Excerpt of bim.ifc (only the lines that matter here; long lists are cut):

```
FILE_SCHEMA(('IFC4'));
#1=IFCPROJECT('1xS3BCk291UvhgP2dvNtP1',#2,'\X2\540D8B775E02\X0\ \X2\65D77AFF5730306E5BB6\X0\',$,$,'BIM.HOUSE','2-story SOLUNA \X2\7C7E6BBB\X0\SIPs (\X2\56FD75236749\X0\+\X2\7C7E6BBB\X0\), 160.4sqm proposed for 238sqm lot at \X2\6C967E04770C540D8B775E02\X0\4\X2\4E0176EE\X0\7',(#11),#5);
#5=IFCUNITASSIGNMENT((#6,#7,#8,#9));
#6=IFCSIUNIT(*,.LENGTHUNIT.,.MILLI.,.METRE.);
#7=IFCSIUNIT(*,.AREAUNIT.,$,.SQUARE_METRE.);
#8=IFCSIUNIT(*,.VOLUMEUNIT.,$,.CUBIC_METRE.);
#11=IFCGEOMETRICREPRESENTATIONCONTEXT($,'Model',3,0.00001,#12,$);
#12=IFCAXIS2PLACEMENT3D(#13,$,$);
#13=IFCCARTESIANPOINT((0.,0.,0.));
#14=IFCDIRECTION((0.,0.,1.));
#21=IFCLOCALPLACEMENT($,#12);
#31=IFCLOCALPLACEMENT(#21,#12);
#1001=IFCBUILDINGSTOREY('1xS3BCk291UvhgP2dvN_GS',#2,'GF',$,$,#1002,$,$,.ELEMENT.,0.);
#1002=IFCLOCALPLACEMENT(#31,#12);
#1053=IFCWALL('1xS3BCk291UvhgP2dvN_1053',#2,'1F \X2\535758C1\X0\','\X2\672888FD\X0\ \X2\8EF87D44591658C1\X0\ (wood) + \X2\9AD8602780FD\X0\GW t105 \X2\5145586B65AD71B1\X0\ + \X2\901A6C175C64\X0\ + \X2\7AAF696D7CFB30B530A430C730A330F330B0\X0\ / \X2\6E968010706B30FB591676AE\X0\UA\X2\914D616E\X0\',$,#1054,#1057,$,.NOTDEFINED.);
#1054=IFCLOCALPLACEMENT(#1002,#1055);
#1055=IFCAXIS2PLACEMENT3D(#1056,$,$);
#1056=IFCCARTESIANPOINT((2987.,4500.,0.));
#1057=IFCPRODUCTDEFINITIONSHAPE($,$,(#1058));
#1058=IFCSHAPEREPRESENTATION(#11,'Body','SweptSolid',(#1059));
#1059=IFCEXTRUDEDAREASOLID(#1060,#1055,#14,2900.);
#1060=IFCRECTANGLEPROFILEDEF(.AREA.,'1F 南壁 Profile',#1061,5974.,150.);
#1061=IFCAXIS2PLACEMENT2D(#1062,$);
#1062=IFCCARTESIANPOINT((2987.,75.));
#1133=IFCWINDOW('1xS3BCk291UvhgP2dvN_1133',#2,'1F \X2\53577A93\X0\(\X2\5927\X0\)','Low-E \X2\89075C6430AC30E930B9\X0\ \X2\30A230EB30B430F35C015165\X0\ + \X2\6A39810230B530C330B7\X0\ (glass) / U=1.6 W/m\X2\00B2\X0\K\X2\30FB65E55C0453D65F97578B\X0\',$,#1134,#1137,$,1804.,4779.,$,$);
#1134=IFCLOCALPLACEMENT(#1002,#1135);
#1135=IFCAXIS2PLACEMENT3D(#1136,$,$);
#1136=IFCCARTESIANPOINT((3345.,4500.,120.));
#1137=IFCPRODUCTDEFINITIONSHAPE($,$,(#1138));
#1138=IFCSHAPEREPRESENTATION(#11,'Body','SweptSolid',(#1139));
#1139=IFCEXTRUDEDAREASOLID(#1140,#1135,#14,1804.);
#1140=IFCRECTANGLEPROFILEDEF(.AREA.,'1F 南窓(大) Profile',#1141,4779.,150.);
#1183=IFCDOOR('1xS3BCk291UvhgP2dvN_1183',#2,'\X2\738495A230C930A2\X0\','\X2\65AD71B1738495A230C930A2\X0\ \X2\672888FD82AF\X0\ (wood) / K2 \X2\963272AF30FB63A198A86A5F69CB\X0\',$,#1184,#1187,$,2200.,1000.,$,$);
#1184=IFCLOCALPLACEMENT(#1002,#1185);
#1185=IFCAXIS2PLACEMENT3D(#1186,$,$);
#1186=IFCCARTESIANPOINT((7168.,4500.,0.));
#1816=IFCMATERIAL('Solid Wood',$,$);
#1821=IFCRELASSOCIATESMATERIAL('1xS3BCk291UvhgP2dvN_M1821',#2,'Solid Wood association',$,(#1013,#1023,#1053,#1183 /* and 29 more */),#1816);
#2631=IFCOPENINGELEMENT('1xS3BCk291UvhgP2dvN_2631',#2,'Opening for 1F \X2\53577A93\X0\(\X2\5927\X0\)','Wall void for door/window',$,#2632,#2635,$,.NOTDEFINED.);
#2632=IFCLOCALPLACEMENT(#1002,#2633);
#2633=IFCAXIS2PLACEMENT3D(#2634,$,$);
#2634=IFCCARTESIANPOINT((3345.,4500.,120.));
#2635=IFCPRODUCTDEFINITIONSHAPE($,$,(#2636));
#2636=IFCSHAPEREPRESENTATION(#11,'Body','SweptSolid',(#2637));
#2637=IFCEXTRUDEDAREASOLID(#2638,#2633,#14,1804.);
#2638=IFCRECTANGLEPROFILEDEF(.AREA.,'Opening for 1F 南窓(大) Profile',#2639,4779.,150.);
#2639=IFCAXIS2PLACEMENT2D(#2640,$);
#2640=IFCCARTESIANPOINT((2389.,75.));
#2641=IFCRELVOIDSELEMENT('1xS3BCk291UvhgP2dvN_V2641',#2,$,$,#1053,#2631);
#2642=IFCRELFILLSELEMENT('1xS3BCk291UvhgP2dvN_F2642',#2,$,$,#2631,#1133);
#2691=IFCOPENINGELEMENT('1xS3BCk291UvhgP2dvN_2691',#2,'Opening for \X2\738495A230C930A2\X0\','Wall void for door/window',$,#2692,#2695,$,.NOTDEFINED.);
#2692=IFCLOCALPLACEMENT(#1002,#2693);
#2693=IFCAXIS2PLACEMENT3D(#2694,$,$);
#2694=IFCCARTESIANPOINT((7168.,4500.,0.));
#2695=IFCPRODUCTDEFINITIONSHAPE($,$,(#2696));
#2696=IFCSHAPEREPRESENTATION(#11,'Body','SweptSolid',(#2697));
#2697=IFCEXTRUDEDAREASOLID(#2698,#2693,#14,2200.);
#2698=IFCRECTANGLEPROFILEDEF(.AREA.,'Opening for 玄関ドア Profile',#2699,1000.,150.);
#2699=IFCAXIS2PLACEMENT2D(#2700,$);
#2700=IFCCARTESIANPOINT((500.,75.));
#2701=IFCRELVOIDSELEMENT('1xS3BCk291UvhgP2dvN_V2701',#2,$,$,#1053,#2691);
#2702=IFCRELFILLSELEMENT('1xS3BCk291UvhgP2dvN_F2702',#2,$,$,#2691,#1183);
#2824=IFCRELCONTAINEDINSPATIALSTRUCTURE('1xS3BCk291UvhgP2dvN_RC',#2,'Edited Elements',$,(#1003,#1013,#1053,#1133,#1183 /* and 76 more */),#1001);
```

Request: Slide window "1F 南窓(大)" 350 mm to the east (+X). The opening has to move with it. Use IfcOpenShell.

```python
import ifcopenshell
import ifcopenshell.api.geometry
import ifcopenshell.util.placement

model = ifcopenshell.open("bim.ifc")

window = model.by_guid("1xS3BCk291UvhgP2dvN_1133")
opening = window.FillsVoids[0].RelatingOpeningElement
wall = opening.VoidsElements[0].RelatingBuildingElement

wall_matrix = ifcopenshell.util.placement.get_local_placement(wall.ObjectPlacement)
shift = wall_matrix[:3, 0] * 350.0
before = ifcopenshell.util.placement.get_local_placement(window.ObjectPlacement)[:3, 3].copy()

# The window is not placed relative to its opening, so move both.
for product in (opening, window):
    matrix = ifcopenshell.util.placement.get_local_placement(product.ObjectPlacement)
    matrix[:3, 3] += shift
    ifcopenshell.api.geometry.edit_object_placement(model, product=product, matrix=matrix, is_si=False)

after = ifcopenshell.util.placement.get_local_placement(window.ObjectPlacement)[:3, 3]
print("window moved by", (after - before).round(3) + 0.0)

model.write("bim-out.ifc")
```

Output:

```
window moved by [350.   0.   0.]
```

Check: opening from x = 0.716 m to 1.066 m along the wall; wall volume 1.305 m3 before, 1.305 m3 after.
